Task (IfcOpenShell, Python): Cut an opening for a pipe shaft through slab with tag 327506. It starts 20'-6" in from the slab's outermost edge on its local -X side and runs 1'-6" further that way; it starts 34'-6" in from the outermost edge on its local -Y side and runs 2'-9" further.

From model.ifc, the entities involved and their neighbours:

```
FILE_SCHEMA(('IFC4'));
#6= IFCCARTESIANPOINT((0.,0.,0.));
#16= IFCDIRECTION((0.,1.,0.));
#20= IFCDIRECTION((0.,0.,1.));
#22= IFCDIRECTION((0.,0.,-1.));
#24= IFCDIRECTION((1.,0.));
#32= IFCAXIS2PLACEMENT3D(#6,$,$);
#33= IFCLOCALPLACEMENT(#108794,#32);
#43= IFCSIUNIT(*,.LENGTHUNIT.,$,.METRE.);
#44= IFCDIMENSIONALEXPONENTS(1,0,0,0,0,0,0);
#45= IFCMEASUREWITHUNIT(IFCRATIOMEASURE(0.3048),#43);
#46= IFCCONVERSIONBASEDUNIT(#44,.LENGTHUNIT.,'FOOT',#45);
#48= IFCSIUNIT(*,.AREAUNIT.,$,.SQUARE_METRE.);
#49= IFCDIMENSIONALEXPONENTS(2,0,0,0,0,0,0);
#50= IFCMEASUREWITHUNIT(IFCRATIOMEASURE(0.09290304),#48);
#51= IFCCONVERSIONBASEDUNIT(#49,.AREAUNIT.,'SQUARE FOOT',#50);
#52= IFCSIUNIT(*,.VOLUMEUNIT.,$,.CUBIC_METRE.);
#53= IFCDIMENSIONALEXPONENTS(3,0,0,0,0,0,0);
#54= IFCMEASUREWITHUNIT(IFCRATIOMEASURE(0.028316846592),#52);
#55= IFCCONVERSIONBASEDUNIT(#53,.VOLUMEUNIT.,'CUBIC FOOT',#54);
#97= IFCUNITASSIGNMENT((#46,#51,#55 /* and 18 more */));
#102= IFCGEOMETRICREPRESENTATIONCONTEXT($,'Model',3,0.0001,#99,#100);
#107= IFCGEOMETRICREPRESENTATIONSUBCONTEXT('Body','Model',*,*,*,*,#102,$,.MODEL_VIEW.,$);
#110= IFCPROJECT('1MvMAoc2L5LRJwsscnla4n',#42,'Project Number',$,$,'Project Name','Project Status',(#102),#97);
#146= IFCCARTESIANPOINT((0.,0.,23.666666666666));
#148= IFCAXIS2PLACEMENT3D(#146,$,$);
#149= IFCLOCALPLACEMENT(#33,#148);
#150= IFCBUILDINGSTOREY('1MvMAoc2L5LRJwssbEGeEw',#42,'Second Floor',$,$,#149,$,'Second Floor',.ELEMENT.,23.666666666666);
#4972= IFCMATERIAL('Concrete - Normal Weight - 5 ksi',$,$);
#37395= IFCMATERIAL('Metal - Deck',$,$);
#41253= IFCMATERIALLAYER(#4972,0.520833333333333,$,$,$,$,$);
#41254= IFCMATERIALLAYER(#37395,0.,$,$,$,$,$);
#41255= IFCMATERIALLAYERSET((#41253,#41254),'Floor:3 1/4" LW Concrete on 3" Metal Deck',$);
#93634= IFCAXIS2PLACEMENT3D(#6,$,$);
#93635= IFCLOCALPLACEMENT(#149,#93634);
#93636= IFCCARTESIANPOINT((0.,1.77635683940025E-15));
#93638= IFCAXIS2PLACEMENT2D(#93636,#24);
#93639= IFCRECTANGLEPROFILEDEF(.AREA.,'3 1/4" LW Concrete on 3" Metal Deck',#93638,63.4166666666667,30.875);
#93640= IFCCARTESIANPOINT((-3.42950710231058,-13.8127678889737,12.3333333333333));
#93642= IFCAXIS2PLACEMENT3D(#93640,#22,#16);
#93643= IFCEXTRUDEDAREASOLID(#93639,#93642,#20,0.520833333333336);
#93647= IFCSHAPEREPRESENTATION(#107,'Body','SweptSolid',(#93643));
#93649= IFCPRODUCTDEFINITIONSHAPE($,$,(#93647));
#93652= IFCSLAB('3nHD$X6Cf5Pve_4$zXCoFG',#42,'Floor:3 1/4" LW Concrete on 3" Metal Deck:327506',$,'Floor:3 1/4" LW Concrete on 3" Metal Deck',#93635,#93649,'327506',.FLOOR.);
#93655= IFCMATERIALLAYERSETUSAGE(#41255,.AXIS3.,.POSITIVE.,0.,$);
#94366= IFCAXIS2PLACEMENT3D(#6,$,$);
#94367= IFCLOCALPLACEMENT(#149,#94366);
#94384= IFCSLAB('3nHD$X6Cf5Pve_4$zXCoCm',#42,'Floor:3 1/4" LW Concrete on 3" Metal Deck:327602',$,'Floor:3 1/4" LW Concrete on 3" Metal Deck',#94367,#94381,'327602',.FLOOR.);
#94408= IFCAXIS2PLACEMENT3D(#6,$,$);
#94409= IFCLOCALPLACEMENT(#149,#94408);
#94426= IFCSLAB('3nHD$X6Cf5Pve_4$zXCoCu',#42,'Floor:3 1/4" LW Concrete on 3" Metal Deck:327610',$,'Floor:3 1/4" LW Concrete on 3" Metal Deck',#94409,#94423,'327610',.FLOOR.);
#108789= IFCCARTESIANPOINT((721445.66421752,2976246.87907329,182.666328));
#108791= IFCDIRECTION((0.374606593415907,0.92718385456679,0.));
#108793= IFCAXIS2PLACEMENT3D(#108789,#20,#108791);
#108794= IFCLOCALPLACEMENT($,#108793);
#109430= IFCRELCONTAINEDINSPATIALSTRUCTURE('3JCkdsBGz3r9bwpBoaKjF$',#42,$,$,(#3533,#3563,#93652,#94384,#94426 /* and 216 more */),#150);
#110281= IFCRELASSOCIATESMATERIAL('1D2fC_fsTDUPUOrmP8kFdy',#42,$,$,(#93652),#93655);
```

```python
import numpy as np
import ifcopenshell
import ifcopenshell.api.feature
import ifcopenshell.api.geometry
import ifcopenshell.api.root
import ifcopenshell.geom
import ifcopenshell.util.placement
import ifcopenshell.util.representation
import ifcopenshell.util.shape
import ifcopenshell.util.unit

model = ifcopenshell.open("model.ifc")
unit_scale = ifcopenshell.util.unit.calculate_unit_scale(model)
settings = ifcopenshell.geom.settings()


def volume(element):
    """Net volume in cubic metres, openings subtracted."""
    shape = ifcopenshell.geom.create_shape(settings, element)
    return ifcopenshell.util.shape.get_volume(shape.geometry)


slab = model.by_guid("3nHD$X6Cf5Pve_4$zXCoFG")
before = volume(slab)

# Extent in the slab's own axes, in metres. The edges named are its -X and -Y sides.
slab_shape = ifcopenshell.geom.create_shape(settings, slab)
vertices = ifcopenshell.util.shape.get_vertices(slab_shape.geometry)
x_min, y_min, bottom = vertices.min(axis=0)
top = vertices[:, 2].max()

opening = ifcopenshell.api.root.create_entity(model, ifc_class="IfcOpeningElement", name="Pipe shaft opening", predefined_type="OPENING")
context = ifcopenshell.util.representation.get_context(model, "Model", "Body", "MODEL_VIEW")
width, depth = 0.4572, 0.8382
outline = [(0.0, 0.0), (width, 0.0), (width, depth), (0.0, depth), (0.0, 0.0)]
# Overshoot both faces by 50 mm so the cut is clean.
shape = ifcopenshell.api.geometry.add_slab_representation(
    model, context=context, depth=top - bottom + 0.1, polyline=outline
)
ifcopenshell.api.geometry.assign_representation(model, product=opening, representation=shape)

matrix = ifcopenshell.util.placement.get_local_placement(slab.ObjectPlacement)
matrix[:, 3] = matrix @ np.append(np.array([x_min + 6.2484, y_min + 10.5156, bottom - 0.05]) / unit_scale, 1.0)
ifcopenshell.api.geometry.edit_object_placement(model, product=opening, matrix=matrix, is_si=False)
ifcopenshell.api.feature.add_feature(model, feature=opening, element=slab)

after = volume(slab)

print(f"slab volume {before:.3f} -> {after:.3f} m3")

model.write("model_updated.ifc")
```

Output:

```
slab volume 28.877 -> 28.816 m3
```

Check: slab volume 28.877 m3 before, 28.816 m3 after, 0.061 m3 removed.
